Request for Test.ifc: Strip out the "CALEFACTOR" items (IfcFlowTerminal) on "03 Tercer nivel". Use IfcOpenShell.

First a look at what the model holds.

```python
import ifcopenshell
import ifcopenshell.util.element

model = ifcopenshell.open("Test.ifc")
print(model.schema)
storey = next(s for s in model.by_type("IfcBuildingStorey") if s.Name == "03 Tercer nivel")
terminals = [e for e in ifcopenshell.util.element.get_decomposition(storey) if e.is_a("IfcFlowTerminal")]
seen = {}
for e in terminals:
    element_type = ifcopenshell.util.element.get_type(e)
    name = element_type.Name if element_type not in (None, e) else None
    seen[name] = seen.get(name, 0) + 1
for name, count in sorted(seen.items(), key=str):
    print(count, "x", name)
```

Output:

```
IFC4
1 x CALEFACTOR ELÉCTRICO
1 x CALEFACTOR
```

```python
import ifcopenshell
import ifcopenshell.api.root
import ifcopenshell.util.element

model = ifcopenshell.open("Test.ifc")

storey = next(s for s in model.by_type("IfcBuildingStorey") if s.Name == "03 Tercer nivel")
terminals = [e for e in ifcopenshell.util.element.get_decomposition(storey) if e.is_a("IfcFlowTerminal")]
targets = [e for e in terminals if (t := ifcopenshell.util.element.get_type(e)) not in (None, e) and t.Name == "CALEFACTOR"]

for e in targets:
    ifcopenshell.api.root.remove_product(model, product=e)
print(len(targets), "removed")

model.write("Test_edited.ifc")
```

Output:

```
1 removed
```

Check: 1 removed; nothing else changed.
